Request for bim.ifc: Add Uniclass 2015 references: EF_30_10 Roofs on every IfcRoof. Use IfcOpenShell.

First a look at what the model holds.

```python
import ifcopenshell

model = ifcopenshell.open("bim.ifc")
print(model.schema)
print("classifications:", [c.Name for c in model.by_type("IfcClassification")])
for ifc_class in ("IfcDoor", "IfcRoof", "IfcStair", "IfcWall", "IfcWindow"):
    print(ifc_class, len(model.by_type(ifc_class)))
```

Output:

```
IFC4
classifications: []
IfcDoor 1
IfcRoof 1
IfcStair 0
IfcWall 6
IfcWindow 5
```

```python
import ifcopenshell
import ifcopenshell.api.classification

model = ifcopenshell.open("bim.ifc")

system = ifcopenshell.api.classification.add_classification(model, classification="Uniclass 2015")

codes = {
    "IfcRoof": ("EF_30_10", "Roofs"),
}
for ifc_class, (code, name) in codes.items():
    products = model.by_type(ifc_class)
    ifcopenshell.api.classification.add_reference(
        model, products=products, classification=system, identification=code, name=name
    )
    print(code, len(products))

model.write("bim_edited.ifc")
```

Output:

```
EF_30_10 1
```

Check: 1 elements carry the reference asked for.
